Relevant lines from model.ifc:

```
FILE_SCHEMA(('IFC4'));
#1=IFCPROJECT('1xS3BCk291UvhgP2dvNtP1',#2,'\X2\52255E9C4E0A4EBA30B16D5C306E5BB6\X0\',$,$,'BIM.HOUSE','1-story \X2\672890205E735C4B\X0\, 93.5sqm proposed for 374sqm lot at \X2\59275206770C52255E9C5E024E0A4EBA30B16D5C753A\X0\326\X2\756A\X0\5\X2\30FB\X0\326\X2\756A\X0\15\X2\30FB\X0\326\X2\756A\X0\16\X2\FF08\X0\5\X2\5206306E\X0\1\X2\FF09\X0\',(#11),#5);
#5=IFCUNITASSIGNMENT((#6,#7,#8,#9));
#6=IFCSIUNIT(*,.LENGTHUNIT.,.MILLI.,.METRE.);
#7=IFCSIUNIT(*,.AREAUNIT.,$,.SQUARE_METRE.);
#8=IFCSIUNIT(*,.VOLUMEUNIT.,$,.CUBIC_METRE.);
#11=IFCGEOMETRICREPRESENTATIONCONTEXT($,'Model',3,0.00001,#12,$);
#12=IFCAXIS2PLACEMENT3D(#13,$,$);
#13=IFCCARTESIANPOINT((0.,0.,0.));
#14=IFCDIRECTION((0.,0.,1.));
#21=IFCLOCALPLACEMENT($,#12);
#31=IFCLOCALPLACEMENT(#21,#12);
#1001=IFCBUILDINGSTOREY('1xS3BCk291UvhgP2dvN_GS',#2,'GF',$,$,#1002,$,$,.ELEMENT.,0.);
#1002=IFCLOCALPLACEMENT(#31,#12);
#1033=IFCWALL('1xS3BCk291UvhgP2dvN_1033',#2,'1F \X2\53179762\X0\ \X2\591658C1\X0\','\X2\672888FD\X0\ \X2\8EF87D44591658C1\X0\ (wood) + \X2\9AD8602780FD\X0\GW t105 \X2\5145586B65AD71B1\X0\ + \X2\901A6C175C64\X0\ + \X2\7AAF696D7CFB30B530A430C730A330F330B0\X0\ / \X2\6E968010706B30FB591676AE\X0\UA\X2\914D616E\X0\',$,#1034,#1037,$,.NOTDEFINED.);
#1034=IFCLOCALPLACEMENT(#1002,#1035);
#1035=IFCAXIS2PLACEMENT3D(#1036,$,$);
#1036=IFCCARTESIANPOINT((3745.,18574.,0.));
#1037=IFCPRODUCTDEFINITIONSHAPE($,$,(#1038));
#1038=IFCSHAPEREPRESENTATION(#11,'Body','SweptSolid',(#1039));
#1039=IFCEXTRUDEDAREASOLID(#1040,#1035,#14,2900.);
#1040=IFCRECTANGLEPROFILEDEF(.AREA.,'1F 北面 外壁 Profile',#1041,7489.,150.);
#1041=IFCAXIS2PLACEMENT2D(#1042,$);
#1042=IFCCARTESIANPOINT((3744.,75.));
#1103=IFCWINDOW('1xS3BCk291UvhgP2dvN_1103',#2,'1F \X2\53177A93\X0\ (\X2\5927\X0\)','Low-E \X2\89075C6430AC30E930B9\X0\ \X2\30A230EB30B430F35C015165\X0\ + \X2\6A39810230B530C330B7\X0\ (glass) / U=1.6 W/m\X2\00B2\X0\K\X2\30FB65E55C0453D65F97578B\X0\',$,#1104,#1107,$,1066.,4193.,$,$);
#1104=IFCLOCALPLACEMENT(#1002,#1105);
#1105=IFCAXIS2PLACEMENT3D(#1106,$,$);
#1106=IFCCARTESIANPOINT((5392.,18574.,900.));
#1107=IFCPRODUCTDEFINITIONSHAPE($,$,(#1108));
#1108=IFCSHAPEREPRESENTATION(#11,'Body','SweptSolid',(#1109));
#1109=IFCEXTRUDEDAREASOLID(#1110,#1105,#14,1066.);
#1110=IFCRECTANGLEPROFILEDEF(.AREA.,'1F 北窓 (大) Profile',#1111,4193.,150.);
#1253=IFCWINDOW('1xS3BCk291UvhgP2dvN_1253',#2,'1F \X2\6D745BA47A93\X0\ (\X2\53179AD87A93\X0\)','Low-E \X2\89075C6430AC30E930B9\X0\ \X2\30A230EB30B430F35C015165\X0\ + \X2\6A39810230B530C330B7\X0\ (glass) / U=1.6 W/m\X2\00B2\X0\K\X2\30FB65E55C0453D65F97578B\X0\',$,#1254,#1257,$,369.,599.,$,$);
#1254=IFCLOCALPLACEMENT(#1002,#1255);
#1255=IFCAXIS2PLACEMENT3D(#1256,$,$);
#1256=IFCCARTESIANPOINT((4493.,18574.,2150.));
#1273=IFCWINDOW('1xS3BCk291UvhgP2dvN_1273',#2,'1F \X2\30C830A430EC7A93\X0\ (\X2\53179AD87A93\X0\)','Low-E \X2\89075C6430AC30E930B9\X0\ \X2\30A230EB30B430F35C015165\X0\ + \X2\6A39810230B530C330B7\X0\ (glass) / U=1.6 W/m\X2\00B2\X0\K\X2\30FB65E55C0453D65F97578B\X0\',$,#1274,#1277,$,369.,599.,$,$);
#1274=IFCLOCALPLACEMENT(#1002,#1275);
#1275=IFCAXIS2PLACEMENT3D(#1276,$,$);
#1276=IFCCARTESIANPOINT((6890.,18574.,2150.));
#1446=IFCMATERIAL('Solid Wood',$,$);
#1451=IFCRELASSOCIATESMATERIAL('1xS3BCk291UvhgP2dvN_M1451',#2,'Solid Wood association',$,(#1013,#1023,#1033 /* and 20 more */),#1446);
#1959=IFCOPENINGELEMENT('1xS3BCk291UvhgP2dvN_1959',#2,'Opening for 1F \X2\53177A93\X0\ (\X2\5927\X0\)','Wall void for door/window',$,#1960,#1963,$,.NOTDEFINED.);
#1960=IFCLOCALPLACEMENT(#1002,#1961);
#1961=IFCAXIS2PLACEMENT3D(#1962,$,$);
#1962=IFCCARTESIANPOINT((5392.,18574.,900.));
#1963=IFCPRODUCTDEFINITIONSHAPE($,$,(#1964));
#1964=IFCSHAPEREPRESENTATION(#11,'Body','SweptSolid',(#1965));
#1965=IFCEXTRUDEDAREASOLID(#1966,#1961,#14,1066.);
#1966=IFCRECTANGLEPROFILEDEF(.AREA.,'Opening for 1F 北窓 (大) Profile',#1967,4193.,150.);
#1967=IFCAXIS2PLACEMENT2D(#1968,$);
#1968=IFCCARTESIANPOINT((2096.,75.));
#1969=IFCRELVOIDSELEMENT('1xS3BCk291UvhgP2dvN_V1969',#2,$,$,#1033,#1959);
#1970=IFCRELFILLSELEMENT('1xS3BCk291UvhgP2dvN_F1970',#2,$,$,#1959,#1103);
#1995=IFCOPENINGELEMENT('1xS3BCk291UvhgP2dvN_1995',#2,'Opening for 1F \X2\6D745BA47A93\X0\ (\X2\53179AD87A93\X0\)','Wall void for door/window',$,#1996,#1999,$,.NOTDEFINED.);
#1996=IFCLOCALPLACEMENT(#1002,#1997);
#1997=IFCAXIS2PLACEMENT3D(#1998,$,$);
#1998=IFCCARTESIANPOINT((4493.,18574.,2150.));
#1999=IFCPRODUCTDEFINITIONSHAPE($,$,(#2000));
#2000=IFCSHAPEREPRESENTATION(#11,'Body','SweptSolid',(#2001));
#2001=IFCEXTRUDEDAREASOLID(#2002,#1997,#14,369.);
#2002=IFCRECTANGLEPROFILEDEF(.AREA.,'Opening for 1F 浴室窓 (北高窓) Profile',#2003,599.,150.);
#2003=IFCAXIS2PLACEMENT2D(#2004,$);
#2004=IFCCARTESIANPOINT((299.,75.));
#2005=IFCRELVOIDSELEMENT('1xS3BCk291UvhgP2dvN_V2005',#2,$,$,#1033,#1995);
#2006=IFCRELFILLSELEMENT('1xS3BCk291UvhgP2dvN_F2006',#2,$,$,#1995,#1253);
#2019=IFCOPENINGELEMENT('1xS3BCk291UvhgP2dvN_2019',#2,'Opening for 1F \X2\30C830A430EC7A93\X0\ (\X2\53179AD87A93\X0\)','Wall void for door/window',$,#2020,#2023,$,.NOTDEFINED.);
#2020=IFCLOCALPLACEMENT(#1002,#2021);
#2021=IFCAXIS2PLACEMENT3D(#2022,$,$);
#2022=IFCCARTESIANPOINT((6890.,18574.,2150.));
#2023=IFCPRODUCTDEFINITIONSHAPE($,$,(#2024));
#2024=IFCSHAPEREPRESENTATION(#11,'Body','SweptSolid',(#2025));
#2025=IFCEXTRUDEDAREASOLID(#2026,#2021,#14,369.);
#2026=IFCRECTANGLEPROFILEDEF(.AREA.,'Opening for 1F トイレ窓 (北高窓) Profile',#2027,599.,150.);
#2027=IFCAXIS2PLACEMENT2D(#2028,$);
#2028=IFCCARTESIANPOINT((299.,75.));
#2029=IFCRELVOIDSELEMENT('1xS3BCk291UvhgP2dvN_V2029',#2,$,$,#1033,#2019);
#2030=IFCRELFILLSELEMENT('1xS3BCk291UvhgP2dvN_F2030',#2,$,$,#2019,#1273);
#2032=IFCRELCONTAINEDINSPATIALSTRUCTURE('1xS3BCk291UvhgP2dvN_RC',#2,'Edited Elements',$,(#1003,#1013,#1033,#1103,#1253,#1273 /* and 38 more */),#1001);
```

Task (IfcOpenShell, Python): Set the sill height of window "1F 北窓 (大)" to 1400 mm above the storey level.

```python
import numpy as np
import ifcopenshell
import ifcopenshell.api.geometry
import ifcopenshell.geom
import ifcopenshell.util.element
import ifcopenshell.util.placement
import ifcopenshell.util.shape
import ifcopenshell.util.unit

model = ifcopenshell.open("model.ifc")
unit_scale = ifcopenshell.util.unit.calculate_unit_scale(model)

window = model.by_guid("1xS3BCk291UvhgP2dvN_1103")
opening = window.FillsVoids[0].RelatingOpeningElement
storey = ifcopenshell.util.element.get_container(window, ifc_class="IfcBuildingStorey")
level = ifcopenshell.util.placement.get_local_placement(storey.ObjectPlacement)[2, 3]

# The opening's origin need not be at the sill, so measure its lowest point.
shape = ifcopenshell.geom.create_shape(ifcopenshell.geom.settings(), opening)
bottom = ifcopenshell.util.shape.get_shape_bottom_elevation(shape, shape.geometry) / unit_scale
dz = level + 1.4 / unit_scale - bottom

shift = np.array([0.0, 0.0, dz])
# The window is not placed relative to its opening, so move both.
for product in (opening, window):
    matrix = ifcopenshell.util.placement.get_local_placement(product.ObjectPlacement)
    matrix[:3, 3] += shift
    ifcopenshell.api.geometry.edit_object_placement(model, product=product, matrix=matrix, is_si=False)

print(f"moved by {dz * unit_scale:+.3f} m")

model.write("model_edited.ifc")
```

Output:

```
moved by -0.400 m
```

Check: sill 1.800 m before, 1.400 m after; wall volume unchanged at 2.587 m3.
